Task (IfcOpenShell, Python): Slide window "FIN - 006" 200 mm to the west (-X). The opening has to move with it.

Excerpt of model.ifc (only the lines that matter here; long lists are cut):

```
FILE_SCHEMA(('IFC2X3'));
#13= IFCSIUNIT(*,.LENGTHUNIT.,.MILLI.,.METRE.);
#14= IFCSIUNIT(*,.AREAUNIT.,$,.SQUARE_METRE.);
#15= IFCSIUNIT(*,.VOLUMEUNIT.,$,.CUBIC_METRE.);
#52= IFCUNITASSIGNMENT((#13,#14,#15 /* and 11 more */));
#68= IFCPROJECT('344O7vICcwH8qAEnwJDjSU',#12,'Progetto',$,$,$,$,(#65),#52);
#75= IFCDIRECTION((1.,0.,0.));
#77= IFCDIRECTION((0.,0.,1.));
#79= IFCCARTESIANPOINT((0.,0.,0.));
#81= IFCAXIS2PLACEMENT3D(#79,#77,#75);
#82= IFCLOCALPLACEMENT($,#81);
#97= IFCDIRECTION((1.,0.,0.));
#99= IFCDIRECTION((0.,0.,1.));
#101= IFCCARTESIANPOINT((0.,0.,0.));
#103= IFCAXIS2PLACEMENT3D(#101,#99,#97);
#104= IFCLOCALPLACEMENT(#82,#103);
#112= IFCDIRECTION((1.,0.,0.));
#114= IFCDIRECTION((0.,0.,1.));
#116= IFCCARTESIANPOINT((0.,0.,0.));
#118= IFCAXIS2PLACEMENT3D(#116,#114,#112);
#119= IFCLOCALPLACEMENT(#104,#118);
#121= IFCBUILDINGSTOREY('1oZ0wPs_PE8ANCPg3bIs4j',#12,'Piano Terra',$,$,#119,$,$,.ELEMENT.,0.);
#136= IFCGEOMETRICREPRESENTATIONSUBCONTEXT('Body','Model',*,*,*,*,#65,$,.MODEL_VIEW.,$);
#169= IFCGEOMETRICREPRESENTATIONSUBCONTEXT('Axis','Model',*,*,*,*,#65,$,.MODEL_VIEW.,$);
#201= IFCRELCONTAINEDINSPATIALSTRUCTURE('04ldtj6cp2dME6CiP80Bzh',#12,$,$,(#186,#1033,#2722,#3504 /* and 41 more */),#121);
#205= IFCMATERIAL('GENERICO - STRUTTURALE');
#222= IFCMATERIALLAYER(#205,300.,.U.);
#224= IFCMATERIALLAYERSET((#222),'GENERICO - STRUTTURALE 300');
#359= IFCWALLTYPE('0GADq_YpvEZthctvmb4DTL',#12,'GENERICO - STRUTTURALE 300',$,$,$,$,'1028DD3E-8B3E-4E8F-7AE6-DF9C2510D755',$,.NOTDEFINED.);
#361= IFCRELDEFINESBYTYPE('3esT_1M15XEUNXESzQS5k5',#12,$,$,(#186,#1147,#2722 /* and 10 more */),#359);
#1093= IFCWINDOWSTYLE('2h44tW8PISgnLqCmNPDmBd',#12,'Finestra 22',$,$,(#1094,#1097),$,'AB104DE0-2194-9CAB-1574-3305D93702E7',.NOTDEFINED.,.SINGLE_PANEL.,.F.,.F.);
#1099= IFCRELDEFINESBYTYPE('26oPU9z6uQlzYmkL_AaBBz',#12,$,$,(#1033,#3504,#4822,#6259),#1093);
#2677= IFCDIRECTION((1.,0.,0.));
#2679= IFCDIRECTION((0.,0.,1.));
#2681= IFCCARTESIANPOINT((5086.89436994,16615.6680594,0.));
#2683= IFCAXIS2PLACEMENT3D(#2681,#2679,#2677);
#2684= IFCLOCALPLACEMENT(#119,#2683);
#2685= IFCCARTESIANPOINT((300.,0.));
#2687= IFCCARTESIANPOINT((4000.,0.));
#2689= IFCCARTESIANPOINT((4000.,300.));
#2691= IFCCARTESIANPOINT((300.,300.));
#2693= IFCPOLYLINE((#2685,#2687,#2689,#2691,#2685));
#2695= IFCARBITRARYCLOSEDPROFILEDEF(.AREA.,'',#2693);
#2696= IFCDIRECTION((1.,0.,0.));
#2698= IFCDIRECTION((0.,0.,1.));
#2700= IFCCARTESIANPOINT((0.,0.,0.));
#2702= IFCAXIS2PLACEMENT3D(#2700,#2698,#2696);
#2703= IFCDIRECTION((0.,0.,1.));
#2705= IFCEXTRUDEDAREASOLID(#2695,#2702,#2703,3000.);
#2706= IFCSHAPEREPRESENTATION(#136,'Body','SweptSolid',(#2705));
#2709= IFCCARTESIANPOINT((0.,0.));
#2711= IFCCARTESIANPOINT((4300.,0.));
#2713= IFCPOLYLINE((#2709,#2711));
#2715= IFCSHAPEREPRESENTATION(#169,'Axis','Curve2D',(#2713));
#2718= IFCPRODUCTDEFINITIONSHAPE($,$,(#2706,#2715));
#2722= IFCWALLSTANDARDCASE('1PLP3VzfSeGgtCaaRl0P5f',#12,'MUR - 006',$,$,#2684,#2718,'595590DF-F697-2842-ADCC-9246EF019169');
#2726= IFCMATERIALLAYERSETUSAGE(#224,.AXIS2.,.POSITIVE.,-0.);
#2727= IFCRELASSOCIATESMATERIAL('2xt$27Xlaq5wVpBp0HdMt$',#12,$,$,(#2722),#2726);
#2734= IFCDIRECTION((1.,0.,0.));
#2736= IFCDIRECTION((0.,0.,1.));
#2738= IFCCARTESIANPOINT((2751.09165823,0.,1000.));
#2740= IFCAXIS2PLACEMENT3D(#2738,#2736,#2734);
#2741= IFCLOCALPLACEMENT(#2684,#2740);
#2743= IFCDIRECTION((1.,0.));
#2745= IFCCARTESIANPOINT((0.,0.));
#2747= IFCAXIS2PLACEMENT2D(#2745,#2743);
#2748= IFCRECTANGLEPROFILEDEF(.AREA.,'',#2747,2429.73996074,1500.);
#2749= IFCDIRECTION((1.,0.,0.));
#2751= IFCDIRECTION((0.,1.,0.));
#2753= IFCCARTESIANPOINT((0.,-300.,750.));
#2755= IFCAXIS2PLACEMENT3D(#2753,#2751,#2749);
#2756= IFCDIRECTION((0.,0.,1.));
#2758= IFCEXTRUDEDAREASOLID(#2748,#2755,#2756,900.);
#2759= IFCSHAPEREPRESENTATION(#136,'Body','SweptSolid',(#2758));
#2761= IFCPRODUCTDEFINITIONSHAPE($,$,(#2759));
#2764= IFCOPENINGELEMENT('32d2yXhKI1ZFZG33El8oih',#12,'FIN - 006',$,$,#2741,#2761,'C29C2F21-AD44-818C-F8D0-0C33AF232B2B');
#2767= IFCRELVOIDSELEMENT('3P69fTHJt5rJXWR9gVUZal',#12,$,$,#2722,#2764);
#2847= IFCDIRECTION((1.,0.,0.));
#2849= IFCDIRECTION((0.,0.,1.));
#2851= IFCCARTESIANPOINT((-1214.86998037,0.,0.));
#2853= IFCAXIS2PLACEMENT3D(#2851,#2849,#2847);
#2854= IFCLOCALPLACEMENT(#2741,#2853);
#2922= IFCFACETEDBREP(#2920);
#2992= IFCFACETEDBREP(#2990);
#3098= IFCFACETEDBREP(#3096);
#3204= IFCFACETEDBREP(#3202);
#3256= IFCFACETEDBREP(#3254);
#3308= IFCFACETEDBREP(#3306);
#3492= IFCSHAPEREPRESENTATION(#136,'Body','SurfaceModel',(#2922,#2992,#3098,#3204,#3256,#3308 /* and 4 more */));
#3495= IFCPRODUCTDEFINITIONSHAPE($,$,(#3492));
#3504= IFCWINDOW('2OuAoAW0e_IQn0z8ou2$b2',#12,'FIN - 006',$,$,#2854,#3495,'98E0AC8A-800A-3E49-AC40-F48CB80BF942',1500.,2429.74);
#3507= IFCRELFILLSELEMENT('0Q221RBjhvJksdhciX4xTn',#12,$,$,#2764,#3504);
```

```python
import ifcopenshell
import ifcopenshell.api.geometry
import ifcopenshell.util.placement
import ifcopenshell.util.unit

model = ifcopenshell.open("model.ifc")
unit_scale = ifcopenshell.util.unit.calculate_unit_scale(model)

window = model.by_guid("2OuAoAW0e_IQn0z8ou2$b2")
opening = window.FillsVoids[0].RelatingOpeningElement
wall = opening.VoidsElements[0].RelatingBuildingElement

wall_matrix = ifcopenshell.util.placement.get_local_placement(wall.ObjectPlacement)
shift = wall_matrix[:3, 0] * -0.2 / unit_scale
before = ifcopenshell.util.placement.get_local_placement(window.ObjectPlacement)[:3, 3].copy()

# The window is placed relative to its opening, so it follows when the opening moves.
matrix = ifcopenshell.util.placement.get_local_placement(opening.ObjectPlacement)
matrix[:3, 3] += shift
ifcopenshell.api.geometry.edit_object_placement(
    model, product=opening, matrix=matrix, is_si=False, should_transform_children=True
)

after = ifcopenshell.util.placement.get_local_placement(window.ObjectPlacement)[:3, 3]
print("window moved by", (after - before).round(3) + 0.0)

model.write("model_updated.ifc")
```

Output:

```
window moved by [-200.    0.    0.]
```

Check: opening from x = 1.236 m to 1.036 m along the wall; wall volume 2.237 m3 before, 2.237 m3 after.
